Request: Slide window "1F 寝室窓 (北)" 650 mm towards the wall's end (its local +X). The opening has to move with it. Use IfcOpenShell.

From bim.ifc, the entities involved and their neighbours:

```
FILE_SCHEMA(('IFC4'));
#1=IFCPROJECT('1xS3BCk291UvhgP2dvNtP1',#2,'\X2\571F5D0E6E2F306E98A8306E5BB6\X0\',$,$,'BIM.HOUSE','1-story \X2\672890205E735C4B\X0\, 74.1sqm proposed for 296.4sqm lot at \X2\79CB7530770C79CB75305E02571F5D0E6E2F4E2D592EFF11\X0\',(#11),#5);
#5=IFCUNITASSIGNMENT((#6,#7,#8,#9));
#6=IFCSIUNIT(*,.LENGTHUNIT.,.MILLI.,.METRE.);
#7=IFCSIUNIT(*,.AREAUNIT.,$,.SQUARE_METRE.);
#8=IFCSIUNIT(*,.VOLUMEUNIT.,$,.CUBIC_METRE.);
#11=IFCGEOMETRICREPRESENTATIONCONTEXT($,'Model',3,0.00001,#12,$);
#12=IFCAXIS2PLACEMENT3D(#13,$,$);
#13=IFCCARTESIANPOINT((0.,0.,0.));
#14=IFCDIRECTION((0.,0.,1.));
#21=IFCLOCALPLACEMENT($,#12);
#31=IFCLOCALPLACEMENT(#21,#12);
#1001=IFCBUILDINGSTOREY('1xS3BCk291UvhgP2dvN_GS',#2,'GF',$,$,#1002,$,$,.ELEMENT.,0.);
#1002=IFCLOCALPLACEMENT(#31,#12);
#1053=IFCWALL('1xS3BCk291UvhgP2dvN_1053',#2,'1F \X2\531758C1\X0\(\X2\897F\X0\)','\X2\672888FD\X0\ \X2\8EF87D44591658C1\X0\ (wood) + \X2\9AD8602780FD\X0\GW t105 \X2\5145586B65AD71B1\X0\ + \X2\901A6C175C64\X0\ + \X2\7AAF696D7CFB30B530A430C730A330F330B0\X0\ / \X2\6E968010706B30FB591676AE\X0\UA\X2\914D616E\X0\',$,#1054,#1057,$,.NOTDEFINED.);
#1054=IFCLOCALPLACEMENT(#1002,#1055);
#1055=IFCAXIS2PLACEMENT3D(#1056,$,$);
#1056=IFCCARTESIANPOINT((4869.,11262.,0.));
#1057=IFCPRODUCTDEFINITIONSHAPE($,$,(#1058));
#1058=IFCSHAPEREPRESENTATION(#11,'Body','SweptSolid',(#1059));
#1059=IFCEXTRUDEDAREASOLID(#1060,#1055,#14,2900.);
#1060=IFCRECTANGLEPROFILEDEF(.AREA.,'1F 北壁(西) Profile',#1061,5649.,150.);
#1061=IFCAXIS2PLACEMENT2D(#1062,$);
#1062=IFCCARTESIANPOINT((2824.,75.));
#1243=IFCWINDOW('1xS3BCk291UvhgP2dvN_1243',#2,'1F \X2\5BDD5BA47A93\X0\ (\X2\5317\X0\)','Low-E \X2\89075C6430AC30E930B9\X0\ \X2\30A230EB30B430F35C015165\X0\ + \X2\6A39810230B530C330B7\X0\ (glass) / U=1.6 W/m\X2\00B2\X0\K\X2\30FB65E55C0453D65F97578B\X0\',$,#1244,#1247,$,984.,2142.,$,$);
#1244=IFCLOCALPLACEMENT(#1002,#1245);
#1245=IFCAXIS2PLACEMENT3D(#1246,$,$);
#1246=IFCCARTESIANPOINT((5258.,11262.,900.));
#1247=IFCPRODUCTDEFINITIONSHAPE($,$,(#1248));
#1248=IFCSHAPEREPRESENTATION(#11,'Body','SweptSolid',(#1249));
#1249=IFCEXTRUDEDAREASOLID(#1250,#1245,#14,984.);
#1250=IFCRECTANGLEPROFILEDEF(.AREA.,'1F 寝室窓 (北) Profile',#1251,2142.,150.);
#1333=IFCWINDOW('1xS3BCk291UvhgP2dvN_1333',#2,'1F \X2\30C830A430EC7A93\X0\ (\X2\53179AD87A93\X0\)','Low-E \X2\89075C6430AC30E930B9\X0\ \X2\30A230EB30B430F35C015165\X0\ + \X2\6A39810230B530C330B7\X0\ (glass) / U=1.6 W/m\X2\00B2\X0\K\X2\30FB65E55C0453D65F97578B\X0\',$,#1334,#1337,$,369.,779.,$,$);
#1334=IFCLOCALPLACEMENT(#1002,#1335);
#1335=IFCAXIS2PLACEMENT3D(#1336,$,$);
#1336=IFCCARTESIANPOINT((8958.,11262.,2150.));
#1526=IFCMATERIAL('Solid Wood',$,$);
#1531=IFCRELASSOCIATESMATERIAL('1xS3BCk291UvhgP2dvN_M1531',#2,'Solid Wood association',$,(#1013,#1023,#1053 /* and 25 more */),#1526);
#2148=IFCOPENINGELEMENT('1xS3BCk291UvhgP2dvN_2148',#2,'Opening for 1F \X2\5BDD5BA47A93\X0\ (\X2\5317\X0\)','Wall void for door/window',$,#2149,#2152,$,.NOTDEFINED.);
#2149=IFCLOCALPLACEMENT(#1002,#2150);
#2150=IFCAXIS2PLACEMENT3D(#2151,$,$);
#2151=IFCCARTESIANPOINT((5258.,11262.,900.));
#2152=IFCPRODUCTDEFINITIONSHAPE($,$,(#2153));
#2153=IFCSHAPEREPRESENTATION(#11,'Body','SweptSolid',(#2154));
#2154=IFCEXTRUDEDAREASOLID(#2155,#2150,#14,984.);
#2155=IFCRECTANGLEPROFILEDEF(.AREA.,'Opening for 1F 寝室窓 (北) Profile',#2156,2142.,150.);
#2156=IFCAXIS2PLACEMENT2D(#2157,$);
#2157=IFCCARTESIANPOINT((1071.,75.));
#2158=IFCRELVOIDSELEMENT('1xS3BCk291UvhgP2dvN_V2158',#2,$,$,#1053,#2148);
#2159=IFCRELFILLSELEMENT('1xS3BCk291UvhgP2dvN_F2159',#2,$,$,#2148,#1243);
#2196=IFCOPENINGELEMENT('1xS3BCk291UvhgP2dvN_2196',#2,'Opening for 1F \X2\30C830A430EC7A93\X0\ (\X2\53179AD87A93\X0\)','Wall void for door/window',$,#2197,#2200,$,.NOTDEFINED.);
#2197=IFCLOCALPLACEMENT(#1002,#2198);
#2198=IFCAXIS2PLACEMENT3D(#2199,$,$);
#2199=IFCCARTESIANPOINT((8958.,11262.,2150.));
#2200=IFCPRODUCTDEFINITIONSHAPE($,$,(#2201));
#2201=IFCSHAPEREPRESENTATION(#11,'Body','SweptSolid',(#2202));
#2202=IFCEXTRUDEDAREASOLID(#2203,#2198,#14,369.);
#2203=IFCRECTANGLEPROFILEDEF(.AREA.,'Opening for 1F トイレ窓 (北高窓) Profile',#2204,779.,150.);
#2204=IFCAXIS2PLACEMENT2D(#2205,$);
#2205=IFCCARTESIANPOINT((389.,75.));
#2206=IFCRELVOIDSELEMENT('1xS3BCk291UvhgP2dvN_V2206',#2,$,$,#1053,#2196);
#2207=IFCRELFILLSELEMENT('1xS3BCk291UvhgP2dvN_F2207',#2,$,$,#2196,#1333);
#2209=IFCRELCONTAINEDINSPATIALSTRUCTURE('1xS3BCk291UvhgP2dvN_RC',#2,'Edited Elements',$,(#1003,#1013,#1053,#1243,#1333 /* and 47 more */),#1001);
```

```python
import ifcopenshell
import ifcopenshell.api.geometry
import ifcopenshell.util.placement

model = ifcopenshell.open("bim.ifc")

window = model.by_id(1243)
opening = window.FillsVoids[0].RelatingOpeningElement
wall = opening.VoidsElements[0].RelatingBuildingElement

wall_matrix = ifcopenshell.util.placement.get_local_placement(wall.ObjectPlacement)
shift = wall_matrix[:3, 0] * 650.0
before = ifcopenshell.util.placement.get_local_placement(window.ObjectPlacement)[:3, 3].copy()

# The window is not placed relative to its opening, so move both.
for product in (opening, window):
    matrix = ifcopenshell.util.placement.get_local_placement(product.ObjectPlacement)
    matrix[:3, 3] += shift
    ifcopenshell.api.geometry.edit_object_placement(model, product=product, matrix=matrix, is_si=False)

after = ifcopenshell.util.placement.get_local_placement(window.ObjectPlacement)[:3, 3]
print("window moved by", (after - before).round(3) + 0.0)

model.write("bim_edited.ifc")
```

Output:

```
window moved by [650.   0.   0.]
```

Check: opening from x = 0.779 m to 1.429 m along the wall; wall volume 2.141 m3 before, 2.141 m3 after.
